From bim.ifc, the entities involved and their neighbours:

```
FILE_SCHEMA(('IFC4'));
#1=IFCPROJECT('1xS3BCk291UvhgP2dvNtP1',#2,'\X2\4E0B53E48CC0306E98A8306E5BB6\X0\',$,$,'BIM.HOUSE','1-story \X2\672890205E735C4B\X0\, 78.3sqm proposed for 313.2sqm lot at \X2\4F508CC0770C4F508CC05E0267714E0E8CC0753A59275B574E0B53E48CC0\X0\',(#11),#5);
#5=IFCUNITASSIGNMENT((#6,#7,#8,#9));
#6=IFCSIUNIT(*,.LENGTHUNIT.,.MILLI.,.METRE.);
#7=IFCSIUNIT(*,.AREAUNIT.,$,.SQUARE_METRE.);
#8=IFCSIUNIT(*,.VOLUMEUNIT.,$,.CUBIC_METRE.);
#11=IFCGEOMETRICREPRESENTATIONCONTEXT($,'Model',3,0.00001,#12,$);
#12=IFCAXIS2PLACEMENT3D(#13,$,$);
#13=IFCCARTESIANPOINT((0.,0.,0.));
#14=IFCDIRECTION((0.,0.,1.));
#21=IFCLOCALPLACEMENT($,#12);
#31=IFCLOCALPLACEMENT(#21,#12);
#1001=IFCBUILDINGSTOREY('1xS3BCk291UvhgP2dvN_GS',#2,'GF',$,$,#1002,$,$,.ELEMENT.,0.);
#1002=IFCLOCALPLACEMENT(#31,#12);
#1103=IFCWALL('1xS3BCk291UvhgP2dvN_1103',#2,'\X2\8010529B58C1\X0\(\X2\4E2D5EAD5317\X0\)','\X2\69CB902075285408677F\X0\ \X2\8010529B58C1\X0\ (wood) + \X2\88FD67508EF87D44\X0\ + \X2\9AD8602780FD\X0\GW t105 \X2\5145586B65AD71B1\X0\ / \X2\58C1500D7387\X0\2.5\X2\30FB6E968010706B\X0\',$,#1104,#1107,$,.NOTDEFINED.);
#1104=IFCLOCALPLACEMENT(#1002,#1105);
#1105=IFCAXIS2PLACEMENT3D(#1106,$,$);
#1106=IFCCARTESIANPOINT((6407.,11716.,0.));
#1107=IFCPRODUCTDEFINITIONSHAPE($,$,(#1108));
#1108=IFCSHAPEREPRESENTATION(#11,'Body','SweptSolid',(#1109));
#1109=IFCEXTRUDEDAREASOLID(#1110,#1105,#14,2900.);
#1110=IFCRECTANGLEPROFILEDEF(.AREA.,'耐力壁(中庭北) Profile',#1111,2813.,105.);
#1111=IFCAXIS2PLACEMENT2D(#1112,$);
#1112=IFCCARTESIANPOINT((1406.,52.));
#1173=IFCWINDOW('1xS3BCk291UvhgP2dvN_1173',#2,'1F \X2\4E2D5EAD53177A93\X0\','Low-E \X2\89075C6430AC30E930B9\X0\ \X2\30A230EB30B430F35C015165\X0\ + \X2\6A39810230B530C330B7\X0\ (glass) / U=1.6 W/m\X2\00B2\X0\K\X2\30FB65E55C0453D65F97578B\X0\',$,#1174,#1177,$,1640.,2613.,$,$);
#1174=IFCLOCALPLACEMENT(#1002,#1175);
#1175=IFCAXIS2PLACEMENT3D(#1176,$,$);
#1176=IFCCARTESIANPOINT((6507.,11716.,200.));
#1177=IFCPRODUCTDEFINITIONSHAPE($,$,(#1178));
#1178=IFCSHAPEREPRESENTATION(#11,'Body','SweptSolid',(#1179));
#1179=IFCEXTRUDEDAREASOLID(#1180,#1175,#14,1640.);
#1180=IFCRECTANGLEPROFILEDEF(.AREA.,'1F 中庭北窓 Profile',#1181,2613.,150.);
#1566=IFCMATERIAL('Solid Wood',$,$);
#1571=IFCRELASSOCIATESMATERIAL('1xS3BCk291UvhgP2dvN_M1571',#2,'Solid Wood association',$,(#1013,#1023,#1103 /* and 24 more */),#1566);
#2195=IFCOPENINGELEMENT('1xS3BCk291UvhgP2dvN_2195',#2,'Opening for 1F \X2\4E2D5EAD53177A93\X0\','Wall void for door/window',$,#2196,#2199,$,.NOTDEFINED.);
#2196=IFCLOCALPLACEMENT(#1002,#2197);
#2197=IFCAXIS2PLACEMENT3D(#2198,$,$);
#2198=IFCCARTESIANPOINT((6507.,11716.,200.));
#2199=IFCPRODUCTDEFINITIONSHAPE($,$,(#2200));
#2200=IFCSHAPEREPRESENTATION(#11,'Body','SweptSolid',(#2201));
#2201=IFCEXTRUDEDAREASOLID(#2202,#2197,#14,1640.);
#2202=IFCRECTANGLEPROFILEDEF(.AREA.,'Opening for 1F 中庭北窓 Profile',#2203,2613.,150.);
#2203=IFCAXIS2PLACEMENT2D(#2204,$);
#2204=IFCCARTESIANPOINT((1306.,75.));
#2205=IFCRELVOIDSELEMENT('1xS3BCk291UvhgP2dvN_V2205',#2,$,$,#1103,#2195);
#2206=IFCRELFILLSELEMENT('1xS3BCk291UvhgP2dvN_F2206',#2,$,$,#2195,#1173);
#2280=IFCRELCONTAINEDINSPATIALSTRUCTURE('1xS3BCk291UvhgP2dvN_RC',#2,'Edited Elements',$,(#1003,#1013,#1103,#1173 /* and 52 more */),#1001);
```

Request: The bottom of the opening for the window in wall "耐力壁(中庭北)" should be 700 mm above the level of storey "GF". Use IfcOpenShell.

```python
import numpy as np
import ifcopenshell
import ifcopenshell.api.geometry
import ifcopenshell.geom
import ifcopenshell.util.element
import ifcopenshell.util.placement
import ifcopenshell.util.shape
import ifcopenshell.util.unit

model = ifcopenshell.open("bim.ifc")
unit_scale = ifcopenshell.util.unit.calculate_unit_scale(model)

window = model.by_guid("1xS3BCk291UvhgP2dvN_1173")
opening = window.FillsVoids[0].RelatingOpeningElement
storey = ifcopenshell.util.element.get_container(window, ifc_class="IfcBuildingStorey")
level = ifcopenshell.util.placement.get_local_placement(storey.ObjectPlacement)[2, 3]

# The opening's origin need not be at the sill, so measure its lowest point.
shape = ifcopenshell.geom.create_shape(ifcopenshell.geom.settings(), opening)
bottom = ifcopenshell.util.shape.get_shape_bottom_elevation(shape, shape.geometry) / unit_scale
dz = level + 700.0 - bottom

shift = np.array([0.0, 0.0, dz])
# The window is not placed relative to its opening, so move both.
for product in (opening, window):
    matrix = ifcopenshell.util.placement.get_local_placement(product.ObjectPlacement)
    matrix[:3, 3] += shift
    ifcopenshell.api.geometry.edit_object_placement(model, product=product, matrix=matrix, is_si=False)

print(f"moved by {dz * unit_scale:+.3f} m")

model.write("bim_updated.ifc")
```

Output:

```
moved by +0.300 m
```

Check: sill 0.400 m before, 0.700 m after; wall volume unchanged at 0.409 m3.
